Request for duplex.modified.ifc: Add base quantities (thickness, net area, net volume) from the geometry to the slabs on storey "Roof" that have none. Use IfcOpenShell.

First a look at what the model holds.

```python
import ifcopenshell
import ifcopenshell.util.element
import ifcopenshell.util.unit

model = ifcopenshell.open("duplex.modified.ifc")
print(model.schema)
for unit_type in ("LENGTHUNIT", "AREAUNIT", "VOLUMEUNIT"):
    print(unit_type, ifcopenshell.util.unit.calculate_unit_scale(model, unit_type))
storey = next(s for s in model.by_type("IfcBuildingStorey") if s.Name == "Roof")
slabs = [e for e in ifcopenshell.util.element.get_decomposition(storey) if e.is_a("IfcSlab")]
for e in sorted(slabs, key=lambda e: e.id()):
    print(e.id(), e.is_a(), e.Name, list(ifcopenshell.util.element.get_psets(e, qtos_only=True)), sep=" | ")
```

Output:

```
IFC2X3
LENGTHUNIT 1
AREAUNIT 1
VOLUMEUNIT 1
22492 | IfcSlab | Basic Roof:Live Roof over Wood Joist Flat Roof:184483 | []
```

```python
import ifcopenshell
import ifcopenshell.api.pset
import ifcopenshell.geom
import ifcopenshell.util.element
import ifcopenshell.util.shape
import ifcopenshell.util.unit

model = ifcopenshell.open("duplex.modified.ifc")
unit_scale = ifcopenshell.util.unit.calculate_unit_scale(model)
area_scale = ifcopenshell.util.unit.calculate_unit_scale(model, "AREAUNIT")
volume_scale = ifcopenshell.util.unit.calculate_unit_scale(model, "VOLUMEUNIT")
settings = ifcopenshell.geom.settings()

storey = next(s for s in model.by_type("IfcBuildingStorey") if s.Name == "Roof")
slabs = [e for e in ifcopenshell.util.element.get_decomposition(storey) if e.is_a("IfcSlab")]

for e in sorted(slabs, key=lambda e: e.id()):
    if ifcopenshell.util.element.get_psets(e, qtos_only=True, should_inherit=False):
        continue
    # Geometry comes back in metres, in the element's own axes.
    shape = ifcopenshell.geom.create_shape(settings, e)
    values = {
        "Width": ifcopenshell.util.shape.get_z(shape.geometry) / unit_scale,
        "NetArea": ifcopenshell.util.shape.get_footprint_area(shape.geometry) / area_scale,
        "NetVolume": ifcopenshell.util.shape.get_volume(shape.geometry) / volume_scale,
    }
    qto = ifcopenshell.api.pset.add_qto(model, product=e, name="BaseQuantities")
    ifcopenshell.api.pset.edit_qto(model, qto=qto, properties=values)
    print(e.id(), {k: round(v, 3) for k, v in values.items()})

model.write("duplex.modified_rev.ifc")
```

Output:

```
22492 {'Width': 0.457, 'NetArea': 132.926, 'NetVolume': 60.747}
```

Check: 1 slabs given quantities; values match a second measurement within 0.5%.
